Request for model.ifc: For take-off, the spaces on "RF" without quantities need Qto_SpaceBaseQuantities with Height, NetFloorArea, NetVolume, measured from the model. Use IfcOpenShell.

First a look at what the model holds.

```python
import ifcopenshell
import ifcopenshell.util.element
import ifcopenshell.util.unit

model = ifcopenshell.open("model.ifc")
print(model.schema)
for unit_type in ("LENGTHUNIT", "AREAUNIT", "VOLUMEUNIT"):
    print(unit_type, ifcopenshell.util.unit.calculate_unit_scale(model, unit_type))
storey = next(s for s in model.by_type("IfcBuildingStorey") if s.Name == "RF")
spaces = [e for e in ifcopenshell.util.element.get_decomposition(storey) if e.is_a("IfcSpace")]
for e in sorted(spaces, key=lambda e: e.id()):
    print(e.id(), e.is_a(), e.Name, list(ifcopenshell.util.element.get_psets(e, qtos_only=True)), sep=" | ")
```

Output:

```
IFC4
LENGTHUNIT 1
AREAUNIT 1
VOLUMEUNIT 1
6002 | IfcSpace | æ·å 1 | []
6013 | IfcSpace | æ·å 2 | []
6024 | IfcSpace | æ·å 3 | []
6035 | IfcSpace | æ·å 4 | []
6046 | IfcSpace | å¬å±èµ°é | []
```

```python
import ifcopenshell
import ifcopenshell.api.pset
import ifcopenshell.geom
import ifcopenshell.util.element
import ifcopenshell.util.shape
import ifcopenshell.util.unit

model = ifcopenshell.open("model.ifc")
unit_scale = ifcopenshell.util.unit.calculate_unit_scale(model)
area_scale = ifcopenshell.util.unit.calculate_unit_scale(model, "AREAUNIT")
volume_scale = ifcopenshell.util.unit.calculate_unit_scale(model, "VOLUMEUNIT")
settings = ifcopenshell.geom.settings()

storey = next(s for s in model.by_type("IfcBuildingStorey") if s.Name == "RF")
spaces = [e for e in ifcopenshell.util.element.get_decomposition(storey) if e.is_a("IfcSpace")]

for e in sorted(spaces, key=lambda e: e.id()):
    if ifcopenshell.util.element.get_psets(e, qtos_only=True, should_inherit=False):
        continue
    # Geometry comes back in metres, in the element's own axes.
    shape = ifcopenshell.geom.create_shape(settings, e)
    values = {
        "Height": ifcopenshell.util.shape.get_z(shape.geometry) / unit_scale,
        "NetFloorArea": ifcopenshell.util.shape.get_footprint_area(shape.geometry) / area_scale,
        "NetVolume": ifcopenshell.util.shape.get_volume(shape.geometry) / volume_scale,
    }
    qto = ifcopenshell.api.pset.add_qto(model, product=e, name="Qto_SpaceBaseQuantities")
    ifcopenshell.api.pset.edit_qto(model, qto=qto, properties=values)
    print(e.id(), {k: round(v, 3) for k, v in values.items()})

model.write("model_v2.ifc")
```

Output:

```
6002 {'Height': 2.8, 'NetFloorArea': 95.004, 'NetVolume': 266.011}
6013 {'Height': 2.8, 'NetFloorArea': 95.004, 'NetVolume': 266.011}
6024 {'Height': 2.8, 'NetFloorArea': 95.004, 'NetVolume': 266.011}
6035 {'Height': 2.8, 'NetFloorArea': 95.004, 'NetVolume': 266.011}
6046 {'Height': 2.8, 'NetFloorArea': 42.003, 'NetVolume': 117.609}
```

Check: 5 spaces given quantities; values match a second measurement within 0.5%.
